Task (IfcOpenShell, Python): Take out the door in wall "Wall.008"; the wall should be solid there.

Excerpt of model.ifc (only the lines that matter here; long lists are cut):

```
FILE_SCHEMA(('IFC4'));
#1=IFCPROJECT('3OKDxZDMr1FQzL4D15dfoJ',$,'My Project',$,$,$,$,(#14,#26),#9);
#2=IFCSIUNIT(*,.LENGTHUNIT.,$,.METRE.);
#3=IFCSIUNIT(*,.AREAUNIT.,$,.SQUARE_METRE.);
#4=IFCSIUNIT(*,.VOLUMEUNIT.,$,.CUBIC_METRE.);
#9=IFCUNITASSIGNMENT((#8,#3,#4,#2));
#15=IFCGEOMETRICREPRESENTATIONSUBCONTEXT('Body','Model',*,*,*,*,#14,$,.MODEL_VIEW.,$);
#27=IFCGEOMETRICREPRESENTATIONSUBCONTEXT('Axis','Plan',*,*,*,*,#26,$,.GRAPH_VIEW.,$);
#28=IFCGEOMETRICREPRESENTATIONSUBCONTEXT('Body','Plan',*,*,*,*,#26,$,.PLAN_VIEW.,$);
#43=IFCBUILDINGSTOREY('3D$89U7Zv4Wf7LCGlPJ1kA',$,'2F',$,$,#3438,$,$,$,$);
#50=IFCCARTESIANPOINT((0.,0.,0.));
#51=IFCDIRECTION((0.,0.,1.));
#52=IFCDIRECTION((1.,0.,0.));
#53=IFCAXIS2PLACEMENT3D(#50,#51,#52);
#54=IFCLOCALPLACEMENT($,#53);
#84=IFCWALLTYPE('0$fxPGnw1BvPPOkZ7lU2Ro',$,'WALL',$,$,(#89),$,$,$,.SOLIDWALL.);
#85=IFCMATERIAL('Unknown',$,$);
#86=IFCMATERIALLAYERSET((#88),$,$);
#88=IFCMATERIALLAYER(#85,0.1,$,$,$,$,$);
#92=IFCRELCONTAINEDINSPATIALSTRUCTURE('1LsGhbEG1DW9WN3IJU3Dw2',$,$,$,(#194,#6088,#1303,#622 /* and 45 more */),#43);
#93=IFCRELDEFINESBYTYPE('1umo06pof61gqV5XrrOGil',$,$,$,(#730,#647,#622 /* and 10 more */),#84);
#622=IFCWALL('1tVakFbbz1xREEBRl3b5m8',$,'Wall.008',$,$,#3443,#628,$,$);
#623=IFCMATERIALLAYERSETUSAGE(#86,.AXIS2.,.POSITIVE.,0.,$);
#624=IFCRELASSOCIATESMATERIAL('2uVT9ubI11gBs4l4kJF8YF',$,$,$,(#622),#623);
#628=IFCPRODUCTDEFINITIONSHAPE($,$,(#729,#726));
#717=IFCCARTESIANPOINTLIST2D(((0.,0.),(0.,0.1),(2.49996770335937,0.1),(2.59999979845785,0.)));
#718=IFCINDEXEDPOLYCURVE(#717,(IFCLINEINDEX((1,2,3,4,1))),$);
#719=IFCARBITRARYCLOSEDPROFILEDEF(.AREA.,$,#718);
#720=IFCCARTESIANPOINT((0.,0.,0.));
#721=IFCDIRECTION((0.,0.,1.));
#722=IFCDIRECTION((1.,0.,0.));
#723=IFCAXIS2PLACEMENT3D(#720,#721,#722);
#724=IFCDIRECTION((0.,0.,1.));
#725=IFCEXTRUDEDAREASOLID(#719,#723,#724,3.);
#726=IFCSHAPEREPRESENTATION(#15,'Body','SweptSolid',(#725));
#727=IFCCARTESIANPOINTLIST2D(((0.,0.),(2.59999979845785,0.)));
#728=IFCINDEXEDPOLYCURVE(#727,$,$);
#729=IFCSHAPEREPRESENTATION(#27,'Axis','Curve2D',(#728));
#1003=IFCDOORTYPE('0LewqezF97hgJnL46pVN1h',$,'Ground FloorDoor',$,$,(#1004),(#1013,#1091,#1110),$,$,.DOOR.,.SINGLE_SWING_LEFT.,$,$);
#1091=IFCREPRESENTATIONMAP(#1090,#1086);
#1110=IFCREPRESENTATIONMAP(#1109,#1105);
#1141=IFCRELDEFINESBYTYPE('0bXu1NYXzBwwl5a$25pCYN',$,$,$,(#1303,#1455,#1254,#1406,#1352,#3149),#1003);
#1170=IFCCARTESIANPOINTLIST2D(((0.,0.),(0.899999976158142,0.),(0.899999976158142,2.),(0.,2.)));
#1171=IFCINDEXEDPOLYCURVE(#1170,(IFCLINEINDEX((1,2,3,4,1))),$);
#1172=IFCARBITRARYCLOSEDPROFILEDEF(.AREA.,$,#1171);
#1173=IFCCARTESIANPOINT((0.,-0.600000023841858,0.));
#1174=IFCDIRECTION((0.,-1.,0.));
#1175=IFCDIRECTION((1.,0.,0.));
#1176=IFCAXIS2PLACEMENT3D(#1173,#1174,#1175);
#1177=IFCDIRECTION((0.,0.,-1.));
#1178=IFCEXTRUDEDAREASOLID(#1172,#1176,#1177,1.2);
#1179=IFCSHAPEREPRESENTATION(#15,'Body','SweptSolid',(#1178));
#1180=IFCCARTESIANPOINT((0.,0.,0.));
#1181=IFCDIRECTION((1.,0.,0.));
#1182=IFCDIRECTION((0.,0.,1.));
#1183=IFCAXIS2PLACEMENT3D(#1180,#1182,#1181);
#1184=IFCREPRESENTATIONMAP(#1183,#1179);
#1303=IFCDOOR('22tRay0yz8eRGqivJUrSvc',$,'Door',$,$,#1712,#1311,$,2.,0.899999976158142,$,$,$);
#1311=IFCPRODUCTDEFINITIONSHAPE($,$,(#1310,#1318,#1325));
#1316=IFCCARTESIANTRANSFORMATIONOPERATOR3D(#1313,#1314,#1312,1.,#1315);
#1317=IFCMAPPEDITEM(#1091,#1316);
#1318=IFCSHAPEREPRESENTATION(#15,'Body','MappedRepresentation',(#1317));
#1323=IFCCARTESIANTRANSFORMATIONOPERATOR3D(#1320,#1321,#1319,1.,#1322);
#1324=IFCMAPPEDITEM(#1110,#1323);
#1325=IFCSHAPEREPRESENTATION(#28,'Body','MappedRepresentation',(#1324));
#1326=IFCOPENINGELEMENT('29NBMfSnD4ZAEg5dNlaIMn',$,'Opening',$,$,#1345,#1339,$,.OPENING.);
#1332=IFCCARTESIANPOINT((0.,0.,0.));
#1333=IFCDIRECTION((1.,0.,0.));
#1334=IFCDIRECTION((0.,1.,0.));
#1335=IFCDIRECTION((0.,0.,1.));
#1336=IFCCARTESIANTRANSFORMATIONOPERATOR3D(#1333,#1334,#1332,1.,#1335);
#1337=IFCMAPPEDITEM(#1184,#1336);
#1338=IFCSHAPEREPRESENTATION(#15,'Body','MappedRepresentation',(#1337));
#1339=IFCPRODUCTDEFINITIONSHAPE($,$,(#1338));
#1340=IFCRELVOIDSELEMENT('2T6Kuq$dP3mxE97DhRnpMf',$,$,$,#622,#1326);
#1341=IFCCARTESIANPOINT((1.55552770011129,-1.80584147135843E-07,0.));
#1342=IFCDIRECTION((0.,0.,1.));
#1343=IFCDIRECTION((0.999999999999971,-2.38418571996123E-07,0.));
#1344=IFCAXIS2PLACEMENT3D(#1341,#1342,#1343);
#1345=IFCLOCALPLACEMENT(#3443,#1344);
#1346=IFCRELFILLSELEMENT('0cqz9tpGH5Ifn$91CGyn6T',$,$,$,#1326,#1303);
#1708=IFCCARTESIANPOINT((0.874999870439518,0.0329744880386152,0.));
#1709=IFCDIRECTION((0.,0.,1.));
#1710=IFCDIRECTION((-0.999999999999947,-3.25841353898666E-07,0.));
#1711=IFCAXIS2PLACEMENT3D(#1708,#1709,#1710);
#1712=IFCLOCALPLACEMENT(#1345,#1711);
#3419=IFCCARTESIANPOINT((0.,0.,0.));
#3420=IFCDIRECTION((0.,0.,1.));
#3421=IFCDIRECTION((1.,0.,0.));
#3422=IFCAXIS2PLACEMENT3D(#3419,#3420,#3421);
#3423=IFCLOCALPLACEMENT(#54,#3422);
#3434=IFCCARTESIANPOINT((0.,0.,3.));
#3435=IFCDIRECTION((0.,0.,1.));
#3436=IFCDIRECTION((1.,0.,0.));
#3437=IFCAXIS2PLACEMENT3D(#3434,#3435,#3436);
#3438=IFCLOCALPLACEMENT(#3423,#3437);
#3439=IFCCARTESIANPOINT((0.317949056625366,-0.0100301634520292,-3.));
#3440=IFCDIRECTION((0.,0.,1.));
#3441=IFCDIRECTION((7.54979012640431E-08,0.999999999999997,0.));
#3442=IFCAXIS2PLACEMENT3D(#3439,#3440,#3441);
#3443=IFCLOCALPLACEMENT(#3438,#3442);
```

```python
import ifcopenshell
import ifcopenshell.api.feature
import ifcopenshell.api.root
import ifcopenshell.geom
import ifcopenshell.util.shape

model = ifcopenshell.open("model.ifc")
settings = ifcopenshell.geom.settings()


def volume(element):
    """Net volume in cubic metres, openings subtracted."""
    shape = ifcopenshell.geom.create_shape(settings, element)
    return ifcopenshell.util.shape.get_volume(shape.geometry)


door = model.by_id(1303)
opening = door.FillsVoids[0].RelatingOpeningElement
wall = opening.VoidsElements[0].RelatingBuildingElement
before = volume(wall)

ifcopenshell.api.root.remove_product(model, product=door)
ifcopenshell.api.feature.remove_feature(model, feature=opening)

after = volume(wall)

print(f"wall volume {before:.3f} -> {after:.3f} m3")

model.write("model_rev.ifc")
```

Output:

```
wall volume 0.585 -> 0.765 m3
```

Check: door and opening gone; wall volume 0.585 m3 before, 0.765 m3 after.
